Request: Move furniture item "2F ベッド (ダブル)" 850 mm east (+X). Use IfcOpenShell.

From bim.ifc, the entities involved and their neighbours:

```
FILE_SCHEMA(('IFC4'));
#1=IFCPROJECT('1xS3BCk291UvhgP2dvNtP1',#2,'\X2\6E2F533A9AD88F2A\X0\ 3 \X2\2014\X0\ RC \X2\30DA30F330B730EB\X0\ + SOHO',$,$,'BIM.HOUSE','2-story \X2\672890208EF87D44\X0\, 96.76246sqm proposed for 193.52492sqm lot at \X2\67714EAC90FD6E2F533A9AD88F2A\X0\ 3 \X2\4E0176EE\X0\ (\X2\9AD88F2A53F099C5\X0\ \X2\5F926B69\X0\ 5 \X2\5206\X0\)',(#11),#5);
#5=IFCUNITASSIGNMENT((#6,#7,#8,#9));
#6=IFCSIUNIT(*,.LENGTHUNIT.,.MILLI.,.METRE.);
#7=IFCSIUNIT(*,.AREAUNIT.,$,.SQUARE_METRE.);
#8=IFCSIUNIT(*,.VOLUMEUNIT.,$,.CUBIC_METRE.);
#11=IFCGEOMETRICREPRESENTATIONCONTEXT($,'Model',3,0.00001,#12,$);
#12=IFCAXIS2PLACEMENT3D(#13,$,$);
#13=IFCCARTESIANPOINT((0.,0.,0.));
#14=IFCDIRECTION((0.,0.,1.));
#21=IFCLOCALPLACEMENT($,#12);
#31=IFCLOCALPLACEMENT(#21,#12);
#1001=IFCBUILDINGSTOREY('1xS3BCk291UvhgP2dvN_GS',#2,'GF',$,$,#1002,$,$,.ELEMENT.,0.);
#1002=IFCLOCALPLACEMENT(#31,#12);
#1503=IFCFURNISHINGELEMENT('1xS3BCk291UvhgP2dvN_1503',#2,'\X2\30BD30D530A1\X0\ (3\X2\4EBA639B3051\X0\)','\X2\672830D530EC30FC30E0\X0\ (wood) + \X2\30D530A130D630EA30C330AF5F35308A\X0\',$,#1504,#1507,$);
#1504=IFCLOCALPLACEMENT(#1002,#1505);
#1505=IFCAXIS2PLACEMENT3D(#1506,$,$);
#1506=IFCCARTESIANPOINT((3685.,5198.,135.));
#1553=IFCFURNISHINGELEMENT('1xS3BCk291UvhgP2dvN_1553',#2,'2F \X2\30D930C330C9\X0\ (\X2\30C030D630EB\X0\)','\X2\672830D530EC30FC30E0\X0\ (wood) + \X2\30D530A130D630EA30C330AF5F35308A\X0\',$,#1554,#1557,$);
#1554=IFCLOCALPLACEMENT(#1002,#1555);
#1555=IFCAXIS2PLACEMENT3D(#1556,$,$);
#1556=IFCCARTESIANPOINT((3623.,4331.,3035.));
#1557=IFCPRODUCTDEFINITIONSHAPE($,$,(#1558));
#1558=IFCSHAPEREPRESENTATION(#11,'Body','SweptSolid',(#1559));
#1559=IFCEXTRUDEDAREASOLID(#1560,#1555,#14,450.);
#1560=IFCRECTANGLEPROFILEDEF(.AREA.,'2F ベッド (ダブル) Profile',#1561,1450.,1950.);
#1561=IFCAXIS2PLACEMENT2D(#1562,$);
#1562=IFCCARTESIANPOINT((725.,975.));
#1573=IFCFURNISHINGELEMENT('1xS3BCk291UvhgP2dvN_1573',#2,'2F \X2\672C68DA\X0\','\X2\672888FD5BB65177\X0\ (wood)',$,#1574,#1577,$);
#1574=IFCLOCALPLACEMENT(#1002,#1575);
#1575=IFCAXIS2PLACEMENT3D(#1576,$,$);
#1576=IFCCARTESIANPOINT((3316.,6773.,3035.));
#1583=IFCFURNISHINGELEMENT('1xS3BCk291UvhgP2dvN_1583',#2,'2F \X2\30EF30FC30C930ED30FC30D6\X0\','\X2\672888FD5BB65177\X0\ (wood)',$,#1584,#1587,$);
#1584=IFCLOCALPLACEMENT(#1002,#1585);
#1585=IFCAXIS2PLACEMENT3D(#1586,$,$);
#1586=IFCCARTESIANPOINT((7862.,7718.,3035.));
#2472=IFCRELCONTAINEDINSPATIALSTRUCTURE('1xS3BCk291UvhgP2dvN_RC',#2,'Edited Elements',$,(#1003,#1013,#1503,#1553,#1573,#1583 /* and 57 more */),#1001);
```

```python
import ifcopenshell
import ifcopenshell.api.geometry
import ifcopenshell.util.placement
import ifcopenshell.util.unit

model = ifcopenshell.open("bim.ifc")
unit_scale = ifcopenshell.util.unit.calculate_unit_scale(model)

item = model.by_guid("1xS3BCk291UvhgP2dvN_1553")
matrix = ifcopenshell.util.placement.get_local_placement(item.ObjectPlacement)
matrix[0, 3] += 0.85 / unit_scale
ifcopenshell.api.geometry.edit_object_placement(model, product=item, matrix=matrix, is_si=False)

print(ifcopenshell.util.placement.get_local_placement(item.ObjectPlacement).round(3) + 0.0)

model.write("bim_edited.ifc")
```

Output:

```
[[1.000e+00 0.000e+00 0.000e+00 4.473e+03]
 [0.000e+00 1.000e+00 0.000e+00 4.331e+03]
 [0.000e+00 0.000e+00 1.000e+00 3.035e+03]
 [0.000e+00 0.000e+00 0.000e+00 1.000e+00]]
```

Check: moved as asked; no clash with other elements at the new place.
